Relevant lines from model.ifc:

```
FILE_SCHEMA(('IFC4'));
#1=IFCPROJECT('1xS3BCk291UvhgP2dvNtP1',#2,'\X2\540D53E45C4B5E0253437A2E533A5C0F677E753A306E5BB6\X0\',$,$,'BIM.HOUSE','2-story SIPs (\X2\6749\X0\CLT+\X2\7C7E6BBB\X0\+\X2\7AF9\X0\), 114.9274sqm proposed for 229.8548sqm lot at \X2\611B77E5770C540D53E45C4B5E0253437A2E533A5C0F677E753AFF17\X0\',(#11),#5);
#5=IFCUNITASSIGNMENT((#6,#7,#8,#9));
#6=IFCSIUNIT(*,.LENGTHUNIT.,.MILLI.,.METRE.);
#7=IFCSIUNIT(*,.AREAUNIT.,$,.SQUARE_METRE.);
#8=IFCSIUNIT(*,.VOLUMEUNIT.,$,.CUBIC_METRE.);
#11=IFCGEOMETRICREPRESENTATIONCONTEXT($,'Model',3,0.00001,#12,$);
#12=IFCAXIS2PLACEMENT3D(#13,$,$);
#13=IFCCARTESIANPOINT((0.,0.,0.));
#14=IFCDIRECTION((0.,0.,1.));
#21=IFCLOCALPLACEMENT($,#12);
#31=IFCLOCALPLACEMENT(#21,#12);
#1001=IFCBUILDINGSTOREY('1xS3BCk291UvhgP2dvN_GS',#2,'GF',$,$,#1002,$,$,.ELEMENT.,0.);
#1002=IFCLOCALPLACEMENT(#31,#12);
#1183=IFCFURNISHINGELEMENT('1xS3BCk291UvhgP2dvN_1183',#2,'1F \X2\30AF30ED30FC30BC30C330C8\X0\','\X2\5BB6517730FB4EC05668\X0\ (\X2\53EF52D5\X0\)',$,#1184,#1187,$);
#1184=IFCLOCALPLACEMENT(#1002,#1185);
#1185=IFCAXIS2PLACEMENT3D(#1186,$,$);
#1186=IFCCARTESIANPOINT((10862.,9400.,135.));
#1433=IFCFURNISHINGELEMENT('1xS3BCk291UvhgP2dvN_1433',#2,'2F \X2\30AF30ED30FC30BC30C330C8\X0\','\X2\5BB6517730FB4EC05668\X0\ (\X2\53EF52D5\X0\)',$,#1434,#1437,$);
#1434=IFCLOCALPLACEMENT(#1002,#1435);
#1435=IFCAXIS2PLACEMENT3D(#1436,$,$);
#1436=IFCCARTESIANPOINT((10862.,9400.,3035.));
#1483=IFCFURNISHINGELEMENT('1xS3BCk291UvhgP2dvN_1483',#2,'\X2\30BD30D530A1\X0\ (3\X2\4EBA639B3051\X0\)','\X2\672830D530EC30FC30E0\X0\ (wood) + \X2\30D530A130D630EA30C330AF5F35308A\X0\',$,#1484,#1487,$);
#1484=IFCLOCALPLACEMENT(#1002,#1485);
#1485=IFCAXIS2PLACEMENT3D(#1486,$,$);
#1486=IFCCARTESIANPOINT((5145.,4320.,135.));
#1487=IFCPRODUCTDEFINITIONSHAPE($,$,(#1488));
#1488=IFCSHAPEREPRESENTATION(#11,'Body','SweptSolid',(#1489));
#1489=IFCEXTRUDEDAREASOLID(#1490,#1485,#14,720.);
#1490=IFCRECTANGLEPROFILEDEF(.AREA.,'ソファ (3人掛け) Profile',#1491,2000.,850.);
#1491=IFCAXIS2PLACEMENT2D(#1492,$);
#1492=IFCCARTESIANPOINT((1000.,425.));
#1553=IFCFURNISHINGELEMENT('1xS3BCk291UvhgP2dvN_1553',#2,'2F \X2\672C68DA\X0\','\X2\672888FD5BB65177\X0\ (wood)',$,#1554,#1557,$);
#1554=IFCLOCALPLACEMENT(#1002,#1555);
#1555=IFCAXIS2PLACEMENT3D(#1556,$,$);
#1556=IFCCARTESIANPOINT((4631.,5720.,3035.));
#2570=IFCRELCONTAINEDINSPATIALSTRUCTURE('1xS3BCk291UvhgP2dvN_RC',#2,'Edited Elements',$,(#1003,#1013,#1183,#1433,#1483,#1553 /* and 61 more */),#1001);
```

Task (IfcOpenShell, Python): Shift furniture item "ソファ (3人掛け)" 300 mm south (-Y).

```python
import ifcopenshell
import ifcopenshell.api.geometry
import ifcopenshell.util.placement
import ifcopenshell.util.unit

model = ifcopenshell.open("model.ifc")
unit_scale = ifcopenshell.util.unit.calculate_unit_scale(model)

item = model.by_guid("1xS3BCk291UvhgP2dvN_1483")
matrix = ifcopenshell.util.placement.get_local_placement(item.ObjectPlacement)
matrix[1, 3] -= 0.3 / unit_scale
ifcopenshell.api.geometry.edit_object_placement(model, product=item, matrix=matrix, is_si=False)

print(ifcopenshell.util.placement.get_local_placement(item.ObjectPlacement).round(3) + 0.0)

model.write("model-out.ifc")
```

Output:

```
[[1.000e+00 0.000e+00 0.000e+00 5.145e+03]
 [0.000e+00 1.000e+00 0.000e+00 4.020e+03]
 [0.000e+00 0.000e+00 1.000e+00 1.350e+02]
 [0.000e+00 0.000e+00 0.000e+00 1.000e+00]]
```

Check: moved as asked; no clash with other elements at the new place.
